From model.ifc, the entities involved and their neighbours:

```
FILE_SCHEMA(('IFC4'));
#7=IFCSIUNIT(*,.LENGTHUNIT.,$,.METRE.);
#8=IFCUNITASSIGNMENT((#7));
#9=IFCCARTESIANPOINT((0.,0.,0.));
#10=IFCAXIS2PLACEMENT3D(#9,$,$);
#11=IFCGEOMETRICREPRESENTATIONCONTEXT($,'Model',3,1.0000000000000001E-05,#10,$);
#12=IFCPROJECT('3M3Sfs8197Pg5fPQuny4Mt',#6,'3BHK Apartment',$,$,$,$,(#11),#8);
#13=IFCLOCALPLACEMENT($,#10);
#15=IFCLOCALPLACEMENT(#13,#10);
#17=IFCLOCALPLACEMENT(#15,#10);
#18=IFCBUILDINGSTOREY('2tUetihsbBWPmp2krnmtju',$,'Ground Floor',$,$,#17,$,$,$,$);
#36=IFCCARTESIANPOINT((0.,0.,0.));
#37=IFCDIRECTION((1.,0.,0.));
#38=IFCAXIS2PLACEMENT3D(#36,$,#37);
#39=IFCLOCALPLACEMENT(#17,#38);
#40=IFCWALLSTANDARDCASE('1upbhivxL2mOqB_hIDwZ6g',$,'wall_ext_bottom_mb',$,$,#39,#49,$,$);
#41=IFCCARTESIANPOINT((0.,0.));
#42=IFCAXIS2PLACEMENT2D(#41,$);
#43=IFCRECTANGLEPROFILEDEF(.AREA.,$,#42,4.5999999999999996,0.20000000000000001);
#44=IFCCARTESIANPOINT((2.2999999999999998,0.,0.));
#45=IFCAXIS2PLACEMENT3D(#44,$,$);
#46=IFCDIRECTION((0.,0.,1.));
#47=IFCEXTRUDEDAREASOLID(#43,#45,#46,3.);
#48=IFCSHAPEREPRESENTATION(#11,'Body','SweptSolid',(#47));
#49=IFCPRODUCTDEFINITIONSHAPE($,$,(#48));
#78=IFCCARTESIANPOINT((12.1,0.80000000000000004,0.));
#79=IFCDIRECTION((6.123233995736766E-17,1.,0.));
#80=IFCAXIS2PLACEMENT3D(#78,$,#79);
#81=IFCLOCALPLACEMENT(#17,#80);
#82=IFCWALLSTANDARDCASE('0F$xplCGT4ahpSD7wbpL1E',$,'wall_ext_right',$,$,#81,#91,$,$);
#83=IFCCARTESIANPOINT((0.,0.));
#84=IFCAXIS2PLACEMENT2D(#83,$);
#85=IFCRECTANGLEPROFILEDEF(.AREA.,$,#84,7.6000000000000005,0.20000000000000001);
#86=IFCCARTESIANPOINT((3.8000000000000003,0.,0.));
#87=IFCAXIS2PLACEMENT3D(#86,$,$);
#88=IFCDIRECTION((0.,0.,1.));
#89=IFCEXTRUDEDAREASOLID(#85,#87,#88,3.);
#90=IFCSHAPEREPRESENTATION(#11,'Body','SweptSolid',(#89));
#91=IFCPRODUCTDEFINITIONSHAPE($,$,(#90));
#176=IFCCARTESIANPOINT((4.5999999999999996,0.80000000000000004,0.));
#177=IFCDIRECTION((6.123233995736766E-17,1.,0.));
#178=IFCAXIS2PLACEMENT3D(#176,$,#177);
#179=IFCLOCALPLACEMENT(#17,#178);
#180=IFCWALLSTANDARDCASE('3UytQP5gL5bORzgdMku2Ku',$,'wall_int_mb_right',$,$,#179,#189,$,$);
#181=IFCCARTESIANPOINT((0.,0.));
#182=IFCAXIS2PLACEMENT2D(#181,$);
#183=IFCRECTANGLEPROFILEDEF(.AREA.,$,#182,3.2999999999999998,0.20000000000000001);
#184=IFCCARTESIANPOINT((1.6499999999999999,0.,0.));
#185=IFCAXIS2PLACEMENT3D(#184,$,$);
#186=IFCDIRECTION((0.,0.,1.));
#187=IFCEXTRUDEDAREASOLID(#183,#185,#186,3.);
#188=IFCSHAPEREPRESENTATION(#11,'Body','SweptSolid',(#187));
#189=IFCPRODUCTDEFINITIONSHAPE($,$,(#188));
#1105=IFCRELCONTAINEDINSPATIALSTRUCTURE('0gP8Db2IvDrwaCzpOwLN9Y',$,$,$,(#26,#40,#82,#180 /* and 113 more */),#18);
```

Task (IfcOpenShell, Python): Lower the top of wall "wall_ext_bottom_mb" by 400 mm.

```python
import ifcopenshell
import ifcopenshell.geom
import ifcopenshell.util.shape

model = ifcopenshell.open("model.ifc")
settings = ifcopenshell.geom.settings()


def volume(element):
    """Net volume in cubic metres, openings subtracted."""
    shape = ifcopenshell.geom.create_shape(settings, element)
    return ifcopenshell.util.shape.get_volume(shape.geometry)


wall = model.by_guid("1upbhivxL2mOqB_hIDwZ6g")
before = volume(wall)

body = next(r for r in wall.Representation.Representations if r.RepresentationIdentifier == "Body")
solid = body.Items[0]
old_height = solid.Depth
solid.Depth -= 0.4
after = volume(wall)

print(f"height {old_height:g} -> {solid.Depth:g}, volume {before:.3f} -> {after:.3f} m3")

model.write("model_updated.ifc")
```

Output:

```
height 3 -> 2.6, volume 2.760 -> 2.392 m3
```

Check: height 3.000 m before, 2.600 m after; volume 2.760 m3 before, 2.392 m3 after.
